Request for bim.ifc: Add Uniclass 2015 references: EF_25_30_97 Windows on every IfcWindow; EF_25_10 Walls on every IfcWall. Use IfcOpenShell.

First a look at what the model holds.

```python
import ifcopenshell

model = ifcopenshell.open("bim.ifc")
print(model.schema)
print("classifications:", [c.Name for c in model.by_type("IfcClassification")])
for ifc_class in ("IfcDoor", "IfcRoof", "IfcStair", "IfcWall", "IfcWindow"):
    print(ifc_class, len(model.by_type(ifc_class)))
```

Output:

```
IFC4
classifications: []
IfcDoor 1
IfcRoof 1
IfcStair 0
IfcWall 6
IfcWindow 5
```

```python
import ifcopenshell
import ifcopenshell.api.classification

model = ifcopenshell.open("bim.ifc")

system = ifcopenshell.api.classification.add_classification(model, classification="Uniclass 2015")

codes = {
    "IfcWindow": ("EF_25_30_97", "Windows"),
    "IfcWall": ("EF_25_10", "Walls"),
}
for ifc_class, (code, name) in codes.items():
    products = model.by_type(ifc_class)
    ifcopenshell.api.classification.add_reference(
        model, products=products, classification=system, identification=code, name=name
    )
    print(code, len(products))

model.write("bim_edited.ifc")
```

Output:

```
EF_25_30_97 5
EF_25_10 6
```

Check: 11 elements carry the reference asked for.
